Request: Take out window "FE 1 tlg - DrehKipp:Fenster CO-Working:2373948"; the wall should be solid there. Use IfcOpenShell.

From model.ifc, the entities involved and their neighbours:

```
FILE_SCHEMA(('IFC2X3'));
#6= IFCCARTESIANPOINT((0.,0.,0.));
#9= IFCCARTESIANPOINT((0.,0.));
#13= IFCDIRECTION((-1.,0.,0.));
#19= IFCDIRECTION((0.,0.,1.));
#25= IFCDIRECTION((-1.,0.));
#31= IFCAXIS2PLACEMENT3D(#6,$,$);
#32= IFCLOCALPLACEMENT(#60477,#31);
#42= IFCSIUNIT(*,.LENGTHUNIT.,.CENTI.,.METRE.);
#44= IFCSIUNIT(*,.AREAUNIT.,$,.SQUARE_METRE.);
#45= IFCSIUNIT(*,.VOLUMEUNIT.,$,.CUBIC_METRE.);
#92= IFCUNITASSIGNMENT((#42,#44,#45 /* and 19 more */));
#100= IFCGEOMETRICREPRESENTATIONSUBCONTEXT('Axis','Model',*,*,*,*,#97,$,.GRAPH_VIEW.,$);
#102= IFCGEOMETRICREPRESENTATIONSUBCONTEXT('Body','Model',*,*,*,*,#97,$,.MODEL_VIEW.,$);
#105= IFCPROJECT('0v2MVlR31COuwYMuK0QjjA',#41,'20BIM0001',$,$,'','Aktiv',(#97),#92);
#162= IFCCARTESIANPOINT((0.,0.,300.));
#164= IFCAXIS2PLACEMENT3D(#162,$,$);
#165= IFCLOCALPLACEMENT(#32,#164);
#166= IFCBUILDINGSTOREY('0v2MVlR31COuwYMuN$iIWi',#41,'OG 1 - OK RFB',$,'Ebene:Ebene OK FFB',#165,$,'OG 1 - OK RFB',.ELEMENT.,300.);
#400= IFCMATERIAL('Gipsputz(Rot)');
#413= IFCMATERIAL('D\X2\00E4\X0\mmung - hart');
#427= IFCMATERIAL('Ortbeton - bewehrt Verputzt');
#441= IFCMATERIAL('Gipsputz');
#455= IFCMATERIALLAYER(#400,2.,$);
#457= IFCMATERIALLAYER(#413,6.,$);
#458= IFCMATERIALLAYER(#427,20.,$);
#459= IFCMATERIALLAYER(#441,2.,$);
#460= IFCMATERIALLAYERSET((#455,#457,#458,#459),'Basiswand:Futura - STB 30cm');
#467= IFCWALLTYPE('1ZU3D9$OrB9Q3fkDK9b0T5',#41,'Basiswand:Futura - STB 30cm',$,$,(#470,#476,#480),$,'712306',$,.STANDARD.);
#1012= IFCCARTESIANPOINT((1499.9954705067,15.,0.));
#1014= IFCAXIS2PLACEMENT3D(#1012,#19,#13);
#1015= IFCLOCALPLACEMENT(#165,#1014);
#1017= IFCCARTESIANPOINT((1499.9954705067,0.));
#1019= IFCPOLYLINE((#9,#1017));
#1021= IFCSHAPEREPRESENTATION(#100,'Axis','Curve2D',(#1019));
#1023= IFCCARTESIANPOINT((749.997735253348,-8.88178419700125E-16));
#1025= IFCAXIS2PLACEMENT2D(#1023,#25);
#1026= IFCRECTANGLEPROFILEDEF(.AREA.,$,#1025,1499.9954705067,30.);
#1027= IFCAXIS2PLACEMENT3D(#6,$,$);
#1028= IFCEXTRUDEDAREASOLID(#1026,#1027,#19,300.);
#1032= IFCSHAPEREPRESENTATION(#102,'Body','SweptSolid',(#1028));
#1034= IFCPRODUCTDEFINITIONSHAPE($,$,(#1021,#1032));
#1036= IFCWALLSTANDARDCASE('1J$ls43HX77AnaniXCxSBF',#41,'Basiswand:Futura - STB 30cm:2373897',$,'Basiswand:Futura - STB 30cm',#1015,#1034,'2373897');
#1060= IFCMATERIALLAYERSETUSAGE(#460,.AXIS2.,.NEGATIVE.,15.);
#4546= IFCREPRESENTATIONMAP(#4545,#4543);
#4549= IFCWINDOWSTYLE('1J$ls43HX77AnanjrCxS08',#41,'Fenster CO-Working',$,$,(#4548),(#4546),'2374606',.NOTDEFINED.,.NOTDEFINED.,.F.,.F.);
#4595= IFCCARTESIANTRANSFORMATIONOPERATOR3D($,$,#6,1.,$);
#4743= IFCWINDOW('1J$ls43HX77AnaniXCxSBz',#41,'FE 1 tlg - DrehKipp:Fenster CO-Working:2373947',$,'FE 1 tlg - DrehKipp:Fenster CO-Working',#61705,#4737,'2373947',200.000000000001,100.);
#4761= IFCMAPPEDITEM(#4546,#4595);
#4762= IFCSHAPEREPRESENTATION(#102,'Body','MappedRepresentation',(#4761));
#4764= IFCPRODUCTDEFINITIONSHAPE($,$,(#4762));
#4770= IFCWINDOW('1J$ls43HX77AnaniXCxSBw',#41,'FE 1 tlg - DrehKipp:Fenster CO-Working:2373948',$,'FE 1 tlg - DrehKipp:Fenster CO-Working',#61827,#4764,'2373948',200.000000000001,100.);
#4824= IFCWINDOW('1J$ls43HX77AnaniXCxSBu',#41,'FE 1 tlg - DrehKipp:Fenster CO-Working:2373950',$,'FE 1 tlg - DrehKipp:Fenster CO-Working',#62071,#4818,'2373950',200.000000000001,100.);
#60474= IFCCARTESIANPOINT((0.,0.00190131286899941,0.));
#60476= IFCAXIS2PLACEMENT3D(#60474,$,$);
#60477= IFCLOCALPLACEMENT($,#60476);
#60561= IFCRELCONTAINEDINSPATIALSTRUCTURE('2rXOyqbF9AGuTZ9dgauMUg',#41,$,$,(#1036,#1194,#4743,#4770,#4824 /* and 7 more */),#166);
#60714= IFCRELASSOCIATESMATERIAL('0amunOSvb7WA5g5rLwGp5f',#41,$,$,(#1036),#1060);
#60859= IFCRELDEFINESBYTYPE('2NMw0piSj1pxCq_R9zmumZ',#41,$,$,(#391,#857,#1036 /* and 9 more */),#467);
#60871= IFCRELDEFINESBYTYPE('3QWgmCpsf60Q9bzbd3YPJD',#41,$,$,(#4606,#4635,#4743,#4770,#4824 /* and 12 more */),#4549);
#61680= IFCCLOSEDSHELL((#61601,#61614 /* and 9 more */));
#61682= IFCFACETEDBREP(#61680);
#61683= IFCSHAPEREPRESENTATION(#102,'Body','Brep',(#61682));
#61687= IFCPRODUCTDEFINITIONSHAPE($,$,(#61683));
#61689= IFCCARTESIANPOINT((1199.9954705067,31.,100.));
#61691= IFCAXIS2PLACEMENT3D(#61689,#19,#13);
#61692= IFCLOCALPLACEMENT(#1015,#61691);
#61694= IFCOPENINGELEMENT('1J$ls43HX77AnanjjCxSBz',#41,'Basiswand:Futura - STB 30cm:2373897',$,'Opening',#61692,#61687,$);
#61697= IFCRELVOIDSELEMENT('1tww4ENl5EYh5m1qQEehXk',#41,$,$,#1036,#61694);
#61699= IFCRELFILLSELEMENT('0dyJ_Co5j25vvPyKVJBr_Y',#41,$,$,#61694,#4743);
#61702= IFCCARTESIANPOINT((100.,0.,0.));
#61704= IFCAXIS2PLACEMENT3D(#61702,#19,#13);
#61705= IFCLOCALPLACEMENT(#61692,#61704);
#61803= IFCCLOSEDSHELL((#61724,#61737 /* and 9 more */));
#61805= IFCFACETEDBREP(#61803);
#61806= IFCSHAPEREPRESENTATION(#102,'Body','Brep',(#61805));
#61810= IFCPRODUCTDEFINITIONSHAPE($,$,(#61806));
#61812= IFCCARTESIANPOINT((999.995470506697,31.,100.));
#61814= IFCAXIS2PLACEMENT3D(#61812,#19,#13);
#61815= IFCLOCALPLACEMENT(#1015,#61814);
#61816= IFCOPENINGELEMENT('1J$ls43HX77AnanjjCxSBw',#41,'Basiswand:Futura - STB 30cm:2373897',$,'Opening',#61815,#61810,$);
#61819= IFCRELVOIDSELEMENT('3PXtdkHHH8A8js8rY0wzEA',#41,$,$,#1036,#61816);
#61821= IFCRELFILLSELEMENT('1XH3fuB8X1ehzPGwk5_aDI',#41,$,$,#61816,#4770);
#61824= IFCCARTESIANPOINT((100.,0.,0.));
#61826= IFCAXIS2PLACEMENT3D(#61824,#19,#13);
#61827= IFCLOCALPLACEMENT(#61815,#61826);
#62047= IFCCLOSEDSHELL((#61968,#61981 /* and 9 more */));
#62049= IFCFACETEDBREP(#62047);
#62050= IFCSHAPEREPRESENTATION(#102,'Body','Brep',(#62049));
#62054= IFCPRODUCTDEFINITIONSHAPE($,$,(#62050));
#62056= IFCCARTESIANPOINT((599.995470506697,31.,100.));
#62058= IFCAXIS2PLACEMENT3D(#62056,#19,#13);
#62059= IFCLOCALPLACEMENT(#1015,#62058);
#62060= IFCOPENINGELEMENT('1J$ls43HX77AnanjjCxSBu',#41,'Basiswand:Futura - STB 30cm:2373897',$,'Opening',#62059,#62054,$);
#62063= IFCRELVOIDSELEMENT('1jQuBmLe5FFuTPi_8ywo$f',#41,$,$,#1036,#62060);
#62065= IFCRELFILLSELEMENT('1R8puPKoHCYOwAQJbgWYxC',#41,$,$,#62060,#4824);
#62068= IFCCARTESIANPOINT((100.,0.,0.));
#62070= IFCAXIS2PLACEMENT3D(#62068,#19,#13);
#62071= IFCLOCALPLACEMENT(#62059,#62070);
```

```python
import ifcopenshell
import ifcopenshell.api.feature
import ifcopenshell.api.root
import ifcopenshell.geom
import ifcopenshell.util.shape

model = ifcopenshell.open("model.ifc")
settings = ifcopenshell.geom.settings()


def volume(element):
    """Net volume in cubic metres, openings subtracted."""
    shape = ifcopenshell.geom.create_shape(settings, element)
    return ifcopenshell.util.shape.get_volume(shape.geometry)


window = model.by_id(4770)
opening = window.FillsVoids[0].RelatingOpeningElement
wall = opening.VoidsElements[0].RelatingBuildingElement
before = volume(wall)

ifcopenshell.api.root.remove_product(model, product=window)
ifcopenshell.api.feature.remove_feature(model, feature=opening)

after = volume(wall)

print(f"wall volume {before:.3f} -> {after:.3f} m3")

model.write("model_v2.ifc")
```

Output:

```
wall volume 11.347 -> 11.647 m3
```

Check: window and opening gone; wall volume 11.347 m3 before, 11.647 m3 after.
